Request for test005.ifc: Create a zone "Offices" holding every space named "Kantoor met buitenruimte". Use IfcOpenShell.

First a look at what the model holds.

```python
import ifcopenshell

model = ifcopenshell.open("test005.ifc")
print(model.schema)
seen = {}
for space in model.by_type("IfcSpace"):
    seen[space.LongName] = seen.get(space.LongName, 0) + 1
for name, count in sorted(seen.items(), key=str):
    print(count, "x", name)
print("zones:", [z.Name for z in model.by_type("IfcZone")][:20])
```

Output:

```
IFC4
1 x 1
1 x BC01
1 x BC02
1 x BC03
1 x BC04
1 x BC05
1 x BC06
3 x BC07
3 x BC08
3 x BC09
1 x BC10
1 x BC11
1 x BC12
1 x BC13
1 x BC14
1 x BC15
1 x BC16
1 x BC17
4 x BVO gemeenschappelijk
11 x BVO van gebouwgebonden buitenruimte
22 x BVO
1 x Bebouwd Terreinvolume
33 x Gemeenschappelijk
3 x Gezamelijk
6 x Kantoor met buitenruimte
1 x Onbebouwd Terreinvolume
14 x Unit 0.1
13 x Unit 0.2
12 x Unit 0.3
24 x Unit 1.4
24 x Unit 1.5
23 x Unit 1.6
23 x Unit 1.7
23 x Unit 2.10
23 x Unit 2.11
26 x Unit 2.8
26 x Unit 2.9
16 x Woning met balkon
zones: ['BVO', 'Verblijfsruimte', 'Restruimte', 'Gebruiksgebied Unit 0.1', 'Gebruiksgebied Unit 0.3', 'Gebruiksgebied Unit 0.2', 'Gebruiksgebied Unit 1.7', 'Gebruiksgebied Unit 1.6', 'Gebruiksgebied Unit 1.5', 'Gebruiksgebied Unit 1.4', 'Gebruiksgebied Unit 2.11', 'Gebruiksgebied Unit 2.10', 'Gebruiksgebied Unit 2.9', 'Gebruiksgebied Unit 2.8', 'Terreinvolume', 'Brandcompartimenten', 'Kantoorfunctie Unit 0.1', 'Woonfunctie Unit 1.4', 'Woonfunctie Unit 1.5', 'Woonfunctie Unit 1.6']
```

```python
import ifcopenshell
import ifcopenshell.api.group
import ifcopenshell.api.root

model = ifcopenshell.open("test005.ifc")

names = {"Kantoor met buitenruimte"}
spaces = [s for s in model.by_type("IfcSpace") if s.LongName in names]

zone = ifcopenshell.api.root.create_entity(model, ifc_class="IfcZone", name="Offices")
ifcopenshell.api.group.assign_group(model, products=spaces, group=zone)
print(len(spaces), "spaces in", zone.Name)

model.write("test005_updated.ifc")
```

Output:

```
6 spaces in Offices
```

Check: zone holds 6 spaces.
